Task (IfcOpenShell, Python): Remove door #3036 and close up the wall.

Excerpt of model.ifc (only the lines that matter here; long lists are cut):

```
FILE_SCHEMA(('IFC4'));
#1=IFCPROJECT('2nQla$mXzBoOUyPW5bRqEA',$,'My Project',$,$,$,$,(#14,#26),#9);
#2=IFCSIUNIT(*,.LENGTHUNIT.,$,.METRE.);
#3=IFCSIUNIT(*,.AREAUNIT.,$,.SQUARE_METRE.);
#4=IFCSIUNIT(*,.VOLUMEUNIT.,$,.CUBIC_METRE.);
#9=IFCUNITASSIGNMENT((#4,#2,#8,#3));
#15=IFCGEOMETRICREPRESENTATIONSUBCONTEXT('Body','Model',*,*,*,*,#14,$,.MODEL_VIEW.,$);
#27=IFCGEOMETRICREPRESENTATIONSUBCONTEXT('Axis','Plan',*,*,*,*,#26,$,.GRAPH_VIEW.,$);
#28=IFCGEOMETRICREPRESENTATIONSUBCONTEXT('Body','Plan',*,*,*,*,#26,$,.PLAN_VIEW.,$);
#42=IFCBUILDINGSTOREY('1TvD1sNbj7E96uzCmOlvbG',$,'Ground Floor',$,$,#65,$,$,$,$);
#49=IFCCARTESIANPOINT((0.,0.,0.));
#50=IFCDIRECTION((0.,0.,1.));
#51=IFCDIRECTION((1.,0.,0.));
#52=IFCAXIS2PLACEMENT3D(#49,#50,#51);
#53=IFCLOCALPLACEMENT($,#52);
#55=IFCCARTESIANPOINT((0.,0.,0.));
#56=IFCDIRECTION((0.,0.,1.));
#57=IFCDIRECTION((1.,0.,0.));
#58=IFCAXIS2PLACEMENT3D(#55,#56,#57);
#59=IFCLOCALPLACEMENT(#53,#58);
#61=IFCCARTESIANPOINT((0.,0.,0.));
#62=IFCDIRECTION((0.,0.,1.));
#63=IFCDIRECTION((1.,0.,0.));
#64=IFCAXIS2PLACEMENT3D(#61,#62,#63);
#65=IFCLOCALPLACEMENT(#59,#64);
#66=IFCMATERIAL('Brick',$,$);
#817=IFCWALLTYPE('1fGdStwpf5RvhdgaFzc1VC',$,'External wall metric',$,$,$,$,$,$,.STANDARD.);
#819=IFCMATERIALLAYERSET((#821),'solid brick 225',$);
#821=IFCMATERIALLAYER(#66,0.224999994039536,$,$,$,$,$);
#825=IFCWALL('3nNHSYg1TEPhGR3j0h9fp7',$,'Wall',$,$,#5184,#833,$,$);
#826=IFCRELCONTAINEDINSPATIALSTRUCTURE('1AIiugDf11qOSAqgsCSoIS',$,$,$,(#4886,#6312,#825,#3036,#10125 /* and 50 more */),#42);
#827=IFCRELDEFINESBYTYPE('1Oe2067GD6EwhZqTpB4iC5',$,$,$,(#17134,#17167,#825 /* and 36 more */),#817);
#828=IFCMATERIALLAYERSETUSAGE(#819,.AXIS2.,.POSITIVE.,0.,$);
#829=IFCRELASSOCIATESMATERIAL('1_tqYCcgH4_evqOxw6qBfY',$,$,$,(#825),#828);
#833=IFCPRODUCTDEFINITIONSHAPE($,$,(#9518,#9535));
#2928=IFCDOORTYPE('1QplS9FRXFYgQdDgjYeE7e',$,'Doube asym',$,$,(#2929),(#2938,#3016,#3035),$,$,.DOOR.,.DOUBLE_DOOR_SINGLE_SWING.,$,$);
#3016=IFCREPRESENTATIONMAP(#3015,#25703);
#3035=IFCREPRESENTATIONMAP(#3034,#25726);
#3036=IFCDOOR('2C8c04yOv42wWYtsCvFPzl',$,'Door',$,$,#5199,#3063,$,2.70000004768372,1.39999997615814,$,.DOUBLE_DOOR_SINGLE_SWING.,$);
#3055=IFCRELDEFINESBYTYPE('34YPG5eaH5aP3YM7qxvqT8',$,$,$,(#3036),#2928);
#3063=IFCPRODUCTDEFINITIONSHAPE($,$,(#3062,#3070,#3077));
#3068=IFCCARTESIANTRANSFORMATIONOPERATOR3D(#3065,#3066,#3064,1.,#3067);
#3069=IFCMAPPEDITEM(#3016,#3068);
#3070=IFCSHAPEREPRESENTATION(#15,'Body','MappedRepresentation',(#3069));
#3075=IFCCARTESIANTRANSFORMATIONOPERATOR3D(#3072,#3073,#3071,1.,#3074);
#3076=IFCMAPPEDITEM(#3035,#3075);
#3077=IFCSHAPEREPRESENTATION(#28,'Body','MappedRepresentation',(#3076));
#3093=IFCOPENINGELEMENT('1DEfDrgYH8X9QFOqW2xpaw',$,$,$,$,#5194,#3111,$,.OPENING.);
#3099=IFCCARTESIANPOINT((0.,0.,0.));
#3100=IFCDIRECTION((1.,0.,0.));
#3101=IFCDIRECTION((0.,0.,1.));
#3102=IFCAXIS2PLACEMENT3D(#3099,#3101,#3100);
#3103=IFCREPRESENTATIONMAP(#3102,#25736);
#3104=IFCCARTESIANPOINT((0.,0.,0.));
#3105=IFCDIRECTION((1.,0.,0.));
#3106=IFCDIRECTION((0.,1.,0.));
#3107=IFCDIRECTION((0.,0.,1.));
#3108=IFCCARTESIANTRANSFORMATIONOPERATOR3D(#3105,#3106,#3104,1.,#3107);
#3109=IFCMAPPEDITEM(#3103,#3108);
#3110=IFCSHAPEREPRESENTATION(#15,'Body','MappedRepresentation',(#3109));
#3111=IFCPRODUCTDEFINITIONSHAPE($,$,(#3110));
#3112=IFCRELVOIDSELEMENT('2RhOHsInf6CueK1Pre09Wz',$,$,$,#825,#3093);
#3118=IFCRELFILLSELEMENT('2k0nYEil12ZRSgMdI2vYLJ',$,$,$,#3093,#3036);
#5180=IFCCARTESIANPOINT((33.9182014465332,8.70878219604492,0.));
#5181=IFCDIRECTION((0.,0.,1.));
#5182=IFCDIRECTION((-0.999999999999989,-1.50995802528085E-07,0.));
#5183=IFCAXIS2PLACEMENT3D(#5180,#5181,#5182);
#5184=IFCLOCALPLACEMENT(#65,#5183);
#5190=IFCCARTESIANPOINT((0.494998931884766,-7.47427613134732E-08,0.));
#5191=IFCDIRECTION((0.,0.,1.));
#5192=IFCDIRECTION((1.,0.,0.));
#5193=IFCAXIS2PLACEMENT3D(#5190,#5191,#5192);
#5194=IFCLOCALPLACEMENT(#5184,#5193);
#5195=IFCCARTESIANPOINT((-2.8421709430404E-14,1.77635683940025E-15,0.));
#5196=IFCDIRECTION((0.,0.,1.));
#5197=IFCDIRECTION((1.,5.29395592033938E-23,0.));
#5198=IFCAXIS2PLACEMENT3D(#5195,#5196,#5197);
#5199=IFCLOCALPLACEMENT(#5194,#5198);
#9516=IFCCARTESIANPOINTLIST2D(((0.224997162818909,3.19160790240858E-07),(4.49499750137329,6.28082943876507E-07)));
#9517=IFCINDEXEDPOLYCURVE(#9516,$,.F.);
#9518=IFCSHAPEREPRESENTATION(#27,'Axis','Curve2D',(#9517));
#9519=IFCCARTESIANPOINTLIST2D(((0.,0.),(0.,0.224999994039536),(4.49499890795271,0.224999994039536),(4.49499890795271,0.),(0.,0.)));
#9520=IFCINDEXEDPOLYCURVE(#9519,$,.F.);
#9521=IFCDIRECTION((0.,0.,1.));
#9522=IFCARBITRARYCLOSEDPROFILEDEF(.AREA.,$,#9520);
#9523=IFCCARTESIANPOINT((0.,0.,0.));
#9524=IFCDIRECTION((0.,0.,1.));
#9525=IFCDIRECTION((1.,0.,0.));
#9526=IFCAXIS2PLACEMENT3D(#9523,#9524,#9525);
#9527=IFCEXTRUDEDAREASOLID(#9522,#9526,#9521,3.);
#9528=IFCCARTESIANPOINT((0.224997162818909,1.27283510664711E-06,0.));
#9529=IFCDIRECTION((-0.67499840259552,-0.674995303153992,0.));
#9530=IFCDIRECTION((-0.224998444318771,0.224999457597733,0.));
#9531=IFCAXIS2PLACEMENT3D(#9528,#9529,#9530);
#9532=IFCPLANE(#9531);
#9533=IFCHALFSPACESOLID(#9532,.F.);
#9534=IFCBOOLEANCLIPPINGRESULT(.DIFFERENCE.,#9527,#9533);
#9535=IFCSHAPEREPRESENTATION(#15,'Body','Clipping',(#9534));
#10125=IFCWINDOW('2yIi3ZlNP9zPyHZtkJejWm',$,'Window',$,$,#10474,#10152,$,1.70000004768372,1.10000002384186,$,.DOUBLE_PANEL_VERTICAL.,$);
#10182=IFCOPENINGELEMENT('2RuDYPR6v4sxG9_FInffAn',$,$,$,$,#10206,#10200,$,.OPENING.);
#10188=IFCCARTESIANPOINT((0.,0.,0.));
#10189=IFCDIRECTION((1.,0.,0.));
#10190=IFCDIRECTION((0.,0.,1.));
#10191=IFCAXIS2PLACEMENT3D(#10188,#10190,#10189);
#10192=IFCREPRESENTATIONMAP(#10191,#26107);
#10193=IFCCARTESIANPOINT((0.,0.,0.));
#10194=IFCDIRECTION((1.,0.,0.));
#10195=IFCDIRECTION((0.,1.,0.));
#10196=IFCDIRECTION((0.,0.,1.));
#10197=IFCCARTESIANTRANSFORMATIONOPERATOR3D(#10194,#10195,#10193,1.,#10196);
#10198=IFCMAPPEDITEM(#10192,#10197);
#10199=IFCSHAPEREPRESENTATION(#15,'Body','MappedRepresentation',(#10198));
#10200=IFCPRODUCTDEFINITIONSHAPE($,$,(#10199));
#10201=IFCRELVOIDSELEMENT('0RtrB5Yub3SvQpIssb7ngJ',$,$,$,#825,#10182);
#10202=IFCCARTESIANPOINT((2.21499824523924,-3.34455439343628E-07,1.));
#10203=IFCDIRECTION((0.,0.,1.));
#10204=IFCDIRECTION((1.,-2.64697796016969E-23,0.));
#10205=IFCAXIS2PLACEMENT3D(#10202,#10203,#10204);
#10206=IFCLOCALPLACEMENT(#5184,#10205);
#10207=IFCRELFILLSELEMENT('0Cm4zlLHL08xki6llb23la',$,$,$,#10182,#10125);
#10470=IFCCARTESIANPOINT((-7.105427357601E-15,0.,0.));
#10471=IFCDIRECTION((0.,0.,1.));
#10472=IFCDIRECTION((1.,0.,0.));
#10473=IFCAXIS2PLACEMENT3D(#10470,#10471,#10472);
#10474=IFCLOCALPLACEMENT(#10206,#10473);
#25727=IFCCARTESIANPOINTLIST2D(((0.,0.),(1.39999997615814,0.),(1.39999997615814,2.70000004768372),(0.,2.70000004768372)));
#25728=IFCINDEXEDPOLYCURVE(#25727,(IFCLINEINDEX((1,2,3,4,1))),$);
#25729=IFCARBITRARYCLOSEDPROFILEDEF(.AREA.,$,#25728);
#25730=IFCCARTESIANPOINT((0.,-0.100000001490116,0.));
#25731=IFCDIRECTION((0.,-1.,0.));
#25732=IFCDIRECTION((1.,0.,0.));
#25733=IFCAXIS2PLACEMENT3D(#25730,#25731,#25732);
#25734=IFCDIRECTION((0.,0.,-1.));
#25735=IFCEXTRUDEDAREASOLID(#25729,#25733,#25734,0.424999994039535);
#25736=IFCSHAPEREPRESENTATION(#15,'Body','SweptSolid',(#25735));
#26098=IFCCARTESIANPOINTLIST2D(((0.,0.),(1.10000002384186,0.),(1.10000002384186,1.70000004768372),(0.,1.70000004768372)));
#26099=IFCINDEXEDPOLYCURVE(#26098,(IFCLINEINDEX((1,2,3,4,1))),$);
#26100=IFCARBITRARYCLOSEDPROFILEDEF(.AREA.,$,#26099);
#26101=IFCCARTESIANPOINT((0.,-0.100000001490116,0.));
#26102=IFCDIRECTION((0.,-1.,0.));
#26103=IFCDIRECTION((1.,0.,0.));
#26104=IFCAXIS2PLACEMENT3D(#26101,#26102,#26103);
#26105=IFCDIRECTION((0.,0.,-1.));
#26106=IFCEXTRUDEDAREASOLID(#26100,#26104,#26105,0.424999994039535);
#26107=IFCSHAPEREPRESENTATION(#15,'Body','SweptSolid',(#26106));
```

```python
import ifcopenshell
import ifcopenshell.api.feature
import ifcopenshell.api.root
import ifcopenshell.geom
import ifcopenshell.util.shape

model = ifcopenshell.open("model.ifc")
settings = ifcopenshell.geom.settings()


def volume(element):
    """Net volume in cubic metres, openings subtracted."""
    shape = ifcopenshell.geom.create_shape(settings, element)
    return ifcopenshell.util.shape.get_volume(shape.geometry)


door = model.by_guid("2C8c04yOv42wWYtsCvFPzl")
opening = door.FillsVoids[0].RelatingOpeningElement
wall = opening.VoidsElements[0].RelatingBuildingElement
before = volume(wall)

ifcopenshell.api.root.remove_product(model, product=door)
ifcopenshell.api.feature.remove_feature(model, feature=opening)

after = volume(wall)

print(f"wall volume {before:.3f} -> {after:.3f} m3")

model.write("model_rev.ifc")
```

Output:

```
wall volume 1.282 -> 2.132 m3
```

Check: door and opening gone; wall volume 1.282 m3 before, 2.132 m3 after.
